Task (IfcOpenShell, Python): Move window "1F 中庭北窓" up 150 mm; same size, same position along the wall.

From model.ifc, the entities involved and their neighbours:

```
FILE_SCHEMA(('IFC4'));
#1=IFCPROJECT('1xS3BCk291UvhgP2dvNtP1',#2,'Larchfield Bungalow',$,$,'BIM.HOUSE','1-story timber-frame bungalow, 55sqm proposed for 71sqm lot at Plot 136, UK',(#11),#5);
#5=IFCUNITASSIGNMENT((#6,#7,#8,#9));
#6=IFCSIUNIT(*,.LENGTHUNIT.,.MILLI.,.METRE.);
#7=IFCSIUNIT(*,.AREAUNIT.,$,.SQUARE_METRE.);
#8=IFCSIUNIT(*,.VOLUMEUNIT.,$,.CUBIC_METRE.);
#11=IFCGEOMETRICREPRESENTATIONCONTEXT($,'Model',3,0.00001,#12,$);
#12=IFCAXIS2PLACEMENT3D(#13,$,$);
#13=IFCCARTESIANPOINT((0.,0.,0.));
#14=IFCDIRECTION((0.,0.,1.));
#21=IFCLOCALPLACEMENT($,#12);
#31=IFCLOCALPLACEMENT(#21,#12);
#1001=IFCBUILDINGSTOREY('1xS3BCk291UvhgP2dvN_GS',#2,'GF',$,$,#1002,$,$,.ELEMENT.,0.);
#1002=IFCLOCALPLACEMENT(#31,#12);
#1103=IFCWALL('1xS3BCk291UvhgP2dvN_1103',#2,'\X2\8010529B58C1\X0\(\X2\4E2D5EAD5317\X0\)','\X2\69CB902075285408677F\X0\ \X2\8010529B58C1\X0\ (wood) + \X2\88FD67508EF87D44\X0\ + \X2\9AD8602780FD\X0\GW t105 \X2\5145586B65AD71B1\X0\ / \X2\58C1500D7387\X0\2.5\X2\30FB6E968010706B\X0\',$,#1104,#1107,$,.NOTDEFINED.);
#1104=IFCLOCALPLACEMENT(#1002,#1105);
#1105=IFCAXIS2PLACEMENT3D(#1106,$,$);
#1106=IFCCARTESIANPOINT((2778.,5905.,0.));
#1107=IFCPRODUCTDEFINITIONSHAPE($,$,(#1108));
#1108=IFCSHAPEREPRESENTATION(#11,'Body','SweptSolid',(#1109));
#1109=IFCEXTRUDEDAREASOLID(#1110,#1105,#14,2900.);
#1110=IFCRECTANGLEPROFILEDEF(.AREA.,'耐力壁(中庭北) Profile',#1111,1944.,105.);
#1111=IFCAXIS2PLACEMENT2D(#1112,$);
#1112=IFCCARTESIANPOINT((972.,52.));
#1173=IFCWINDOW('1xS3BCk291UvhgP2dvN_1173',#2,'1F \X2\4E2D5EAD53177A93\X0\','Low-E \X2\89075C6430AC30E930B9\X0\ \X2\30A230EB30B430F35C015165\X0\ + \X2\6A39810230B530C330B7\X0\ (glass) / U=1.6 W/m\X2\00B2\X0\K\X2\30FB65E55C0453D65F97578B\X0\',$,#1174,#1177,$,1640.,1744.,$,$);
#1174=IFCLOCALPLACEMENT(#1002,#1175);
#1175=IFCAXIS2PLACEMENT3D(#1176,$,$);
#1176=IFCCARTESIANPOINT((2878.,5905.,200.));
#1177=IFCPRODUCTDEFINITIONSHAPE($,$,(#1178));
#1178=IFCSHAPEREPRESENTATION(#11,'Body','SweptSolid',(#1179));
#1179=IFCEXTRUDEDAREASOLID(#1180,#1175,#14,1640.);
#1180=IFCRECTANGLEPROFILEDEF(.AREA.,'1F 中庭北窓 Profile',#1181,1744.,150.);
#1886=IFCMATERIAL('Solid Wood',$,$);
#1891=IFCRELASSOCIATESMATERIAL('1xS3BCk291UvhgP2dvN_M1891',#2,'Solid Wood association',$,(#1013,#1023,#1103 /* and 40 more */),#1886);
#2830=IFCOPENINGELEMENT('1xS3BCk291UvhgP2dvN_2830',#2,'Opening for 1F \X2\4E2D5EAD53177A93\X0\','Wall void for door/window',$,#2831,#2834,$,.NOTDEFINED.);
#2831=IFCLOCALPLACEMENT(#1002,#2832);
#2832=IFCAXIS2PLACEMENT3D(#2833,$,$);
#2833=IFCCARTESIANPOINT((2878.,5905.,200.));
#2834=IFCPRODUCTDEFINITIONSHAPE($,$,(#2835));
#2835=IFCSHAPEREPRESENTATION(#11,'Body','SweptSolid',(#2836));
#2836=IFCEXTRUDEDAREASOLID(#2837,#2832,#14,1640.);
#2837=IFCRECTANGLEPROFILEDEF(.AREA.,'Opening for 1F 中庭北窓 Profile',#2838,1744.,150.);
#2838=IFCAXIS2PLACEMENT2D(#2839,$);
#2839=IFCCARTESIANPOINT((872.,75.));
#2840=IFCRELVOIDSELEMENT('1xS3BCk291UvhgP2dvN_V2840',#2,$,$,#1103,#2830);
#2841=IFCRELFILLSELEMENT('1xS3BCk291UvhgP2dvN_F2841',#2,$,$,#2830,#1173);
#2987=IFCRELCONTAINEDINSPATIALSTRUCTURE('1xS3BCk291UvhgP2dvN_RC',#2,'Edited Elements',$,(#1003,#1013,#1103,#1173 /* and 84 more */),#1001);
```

```python
import numpy as np
import ifcopenshell
import ifcopenshell.api.geometry
import ifcopenshell.util.placement
import ifcopenshell.util.unit

model = ifcopenshell.open("model.ifc")
unit_scale = ifcopenshell.util.unit.calculate_unit_scale(model)

window = model.by_id(1173)
opening = window.FillsVoids[0].RelatingOpeningElement
dz = 0.15 / unit_scale

shift = np.array([0.0, 0.0, dz])
# The window is not placed relative to its opening, so move both.
for product in (opening, window):
    matrix = ifcopenshell.util.placement.get_local_placement(product.ObjectPlacement)
    matrix[:3, 3] += shift
    ifcopenshell.api.geometry.edit_object_placement(model, product=product, matrix=matrix, is_si=False)

print(f"moved by {dz * unit_scale:+.3f} m")

model.write("model_edited.ifc")
```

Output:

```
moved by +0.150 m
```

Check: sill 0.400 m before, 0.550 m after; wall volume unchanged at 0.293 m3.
